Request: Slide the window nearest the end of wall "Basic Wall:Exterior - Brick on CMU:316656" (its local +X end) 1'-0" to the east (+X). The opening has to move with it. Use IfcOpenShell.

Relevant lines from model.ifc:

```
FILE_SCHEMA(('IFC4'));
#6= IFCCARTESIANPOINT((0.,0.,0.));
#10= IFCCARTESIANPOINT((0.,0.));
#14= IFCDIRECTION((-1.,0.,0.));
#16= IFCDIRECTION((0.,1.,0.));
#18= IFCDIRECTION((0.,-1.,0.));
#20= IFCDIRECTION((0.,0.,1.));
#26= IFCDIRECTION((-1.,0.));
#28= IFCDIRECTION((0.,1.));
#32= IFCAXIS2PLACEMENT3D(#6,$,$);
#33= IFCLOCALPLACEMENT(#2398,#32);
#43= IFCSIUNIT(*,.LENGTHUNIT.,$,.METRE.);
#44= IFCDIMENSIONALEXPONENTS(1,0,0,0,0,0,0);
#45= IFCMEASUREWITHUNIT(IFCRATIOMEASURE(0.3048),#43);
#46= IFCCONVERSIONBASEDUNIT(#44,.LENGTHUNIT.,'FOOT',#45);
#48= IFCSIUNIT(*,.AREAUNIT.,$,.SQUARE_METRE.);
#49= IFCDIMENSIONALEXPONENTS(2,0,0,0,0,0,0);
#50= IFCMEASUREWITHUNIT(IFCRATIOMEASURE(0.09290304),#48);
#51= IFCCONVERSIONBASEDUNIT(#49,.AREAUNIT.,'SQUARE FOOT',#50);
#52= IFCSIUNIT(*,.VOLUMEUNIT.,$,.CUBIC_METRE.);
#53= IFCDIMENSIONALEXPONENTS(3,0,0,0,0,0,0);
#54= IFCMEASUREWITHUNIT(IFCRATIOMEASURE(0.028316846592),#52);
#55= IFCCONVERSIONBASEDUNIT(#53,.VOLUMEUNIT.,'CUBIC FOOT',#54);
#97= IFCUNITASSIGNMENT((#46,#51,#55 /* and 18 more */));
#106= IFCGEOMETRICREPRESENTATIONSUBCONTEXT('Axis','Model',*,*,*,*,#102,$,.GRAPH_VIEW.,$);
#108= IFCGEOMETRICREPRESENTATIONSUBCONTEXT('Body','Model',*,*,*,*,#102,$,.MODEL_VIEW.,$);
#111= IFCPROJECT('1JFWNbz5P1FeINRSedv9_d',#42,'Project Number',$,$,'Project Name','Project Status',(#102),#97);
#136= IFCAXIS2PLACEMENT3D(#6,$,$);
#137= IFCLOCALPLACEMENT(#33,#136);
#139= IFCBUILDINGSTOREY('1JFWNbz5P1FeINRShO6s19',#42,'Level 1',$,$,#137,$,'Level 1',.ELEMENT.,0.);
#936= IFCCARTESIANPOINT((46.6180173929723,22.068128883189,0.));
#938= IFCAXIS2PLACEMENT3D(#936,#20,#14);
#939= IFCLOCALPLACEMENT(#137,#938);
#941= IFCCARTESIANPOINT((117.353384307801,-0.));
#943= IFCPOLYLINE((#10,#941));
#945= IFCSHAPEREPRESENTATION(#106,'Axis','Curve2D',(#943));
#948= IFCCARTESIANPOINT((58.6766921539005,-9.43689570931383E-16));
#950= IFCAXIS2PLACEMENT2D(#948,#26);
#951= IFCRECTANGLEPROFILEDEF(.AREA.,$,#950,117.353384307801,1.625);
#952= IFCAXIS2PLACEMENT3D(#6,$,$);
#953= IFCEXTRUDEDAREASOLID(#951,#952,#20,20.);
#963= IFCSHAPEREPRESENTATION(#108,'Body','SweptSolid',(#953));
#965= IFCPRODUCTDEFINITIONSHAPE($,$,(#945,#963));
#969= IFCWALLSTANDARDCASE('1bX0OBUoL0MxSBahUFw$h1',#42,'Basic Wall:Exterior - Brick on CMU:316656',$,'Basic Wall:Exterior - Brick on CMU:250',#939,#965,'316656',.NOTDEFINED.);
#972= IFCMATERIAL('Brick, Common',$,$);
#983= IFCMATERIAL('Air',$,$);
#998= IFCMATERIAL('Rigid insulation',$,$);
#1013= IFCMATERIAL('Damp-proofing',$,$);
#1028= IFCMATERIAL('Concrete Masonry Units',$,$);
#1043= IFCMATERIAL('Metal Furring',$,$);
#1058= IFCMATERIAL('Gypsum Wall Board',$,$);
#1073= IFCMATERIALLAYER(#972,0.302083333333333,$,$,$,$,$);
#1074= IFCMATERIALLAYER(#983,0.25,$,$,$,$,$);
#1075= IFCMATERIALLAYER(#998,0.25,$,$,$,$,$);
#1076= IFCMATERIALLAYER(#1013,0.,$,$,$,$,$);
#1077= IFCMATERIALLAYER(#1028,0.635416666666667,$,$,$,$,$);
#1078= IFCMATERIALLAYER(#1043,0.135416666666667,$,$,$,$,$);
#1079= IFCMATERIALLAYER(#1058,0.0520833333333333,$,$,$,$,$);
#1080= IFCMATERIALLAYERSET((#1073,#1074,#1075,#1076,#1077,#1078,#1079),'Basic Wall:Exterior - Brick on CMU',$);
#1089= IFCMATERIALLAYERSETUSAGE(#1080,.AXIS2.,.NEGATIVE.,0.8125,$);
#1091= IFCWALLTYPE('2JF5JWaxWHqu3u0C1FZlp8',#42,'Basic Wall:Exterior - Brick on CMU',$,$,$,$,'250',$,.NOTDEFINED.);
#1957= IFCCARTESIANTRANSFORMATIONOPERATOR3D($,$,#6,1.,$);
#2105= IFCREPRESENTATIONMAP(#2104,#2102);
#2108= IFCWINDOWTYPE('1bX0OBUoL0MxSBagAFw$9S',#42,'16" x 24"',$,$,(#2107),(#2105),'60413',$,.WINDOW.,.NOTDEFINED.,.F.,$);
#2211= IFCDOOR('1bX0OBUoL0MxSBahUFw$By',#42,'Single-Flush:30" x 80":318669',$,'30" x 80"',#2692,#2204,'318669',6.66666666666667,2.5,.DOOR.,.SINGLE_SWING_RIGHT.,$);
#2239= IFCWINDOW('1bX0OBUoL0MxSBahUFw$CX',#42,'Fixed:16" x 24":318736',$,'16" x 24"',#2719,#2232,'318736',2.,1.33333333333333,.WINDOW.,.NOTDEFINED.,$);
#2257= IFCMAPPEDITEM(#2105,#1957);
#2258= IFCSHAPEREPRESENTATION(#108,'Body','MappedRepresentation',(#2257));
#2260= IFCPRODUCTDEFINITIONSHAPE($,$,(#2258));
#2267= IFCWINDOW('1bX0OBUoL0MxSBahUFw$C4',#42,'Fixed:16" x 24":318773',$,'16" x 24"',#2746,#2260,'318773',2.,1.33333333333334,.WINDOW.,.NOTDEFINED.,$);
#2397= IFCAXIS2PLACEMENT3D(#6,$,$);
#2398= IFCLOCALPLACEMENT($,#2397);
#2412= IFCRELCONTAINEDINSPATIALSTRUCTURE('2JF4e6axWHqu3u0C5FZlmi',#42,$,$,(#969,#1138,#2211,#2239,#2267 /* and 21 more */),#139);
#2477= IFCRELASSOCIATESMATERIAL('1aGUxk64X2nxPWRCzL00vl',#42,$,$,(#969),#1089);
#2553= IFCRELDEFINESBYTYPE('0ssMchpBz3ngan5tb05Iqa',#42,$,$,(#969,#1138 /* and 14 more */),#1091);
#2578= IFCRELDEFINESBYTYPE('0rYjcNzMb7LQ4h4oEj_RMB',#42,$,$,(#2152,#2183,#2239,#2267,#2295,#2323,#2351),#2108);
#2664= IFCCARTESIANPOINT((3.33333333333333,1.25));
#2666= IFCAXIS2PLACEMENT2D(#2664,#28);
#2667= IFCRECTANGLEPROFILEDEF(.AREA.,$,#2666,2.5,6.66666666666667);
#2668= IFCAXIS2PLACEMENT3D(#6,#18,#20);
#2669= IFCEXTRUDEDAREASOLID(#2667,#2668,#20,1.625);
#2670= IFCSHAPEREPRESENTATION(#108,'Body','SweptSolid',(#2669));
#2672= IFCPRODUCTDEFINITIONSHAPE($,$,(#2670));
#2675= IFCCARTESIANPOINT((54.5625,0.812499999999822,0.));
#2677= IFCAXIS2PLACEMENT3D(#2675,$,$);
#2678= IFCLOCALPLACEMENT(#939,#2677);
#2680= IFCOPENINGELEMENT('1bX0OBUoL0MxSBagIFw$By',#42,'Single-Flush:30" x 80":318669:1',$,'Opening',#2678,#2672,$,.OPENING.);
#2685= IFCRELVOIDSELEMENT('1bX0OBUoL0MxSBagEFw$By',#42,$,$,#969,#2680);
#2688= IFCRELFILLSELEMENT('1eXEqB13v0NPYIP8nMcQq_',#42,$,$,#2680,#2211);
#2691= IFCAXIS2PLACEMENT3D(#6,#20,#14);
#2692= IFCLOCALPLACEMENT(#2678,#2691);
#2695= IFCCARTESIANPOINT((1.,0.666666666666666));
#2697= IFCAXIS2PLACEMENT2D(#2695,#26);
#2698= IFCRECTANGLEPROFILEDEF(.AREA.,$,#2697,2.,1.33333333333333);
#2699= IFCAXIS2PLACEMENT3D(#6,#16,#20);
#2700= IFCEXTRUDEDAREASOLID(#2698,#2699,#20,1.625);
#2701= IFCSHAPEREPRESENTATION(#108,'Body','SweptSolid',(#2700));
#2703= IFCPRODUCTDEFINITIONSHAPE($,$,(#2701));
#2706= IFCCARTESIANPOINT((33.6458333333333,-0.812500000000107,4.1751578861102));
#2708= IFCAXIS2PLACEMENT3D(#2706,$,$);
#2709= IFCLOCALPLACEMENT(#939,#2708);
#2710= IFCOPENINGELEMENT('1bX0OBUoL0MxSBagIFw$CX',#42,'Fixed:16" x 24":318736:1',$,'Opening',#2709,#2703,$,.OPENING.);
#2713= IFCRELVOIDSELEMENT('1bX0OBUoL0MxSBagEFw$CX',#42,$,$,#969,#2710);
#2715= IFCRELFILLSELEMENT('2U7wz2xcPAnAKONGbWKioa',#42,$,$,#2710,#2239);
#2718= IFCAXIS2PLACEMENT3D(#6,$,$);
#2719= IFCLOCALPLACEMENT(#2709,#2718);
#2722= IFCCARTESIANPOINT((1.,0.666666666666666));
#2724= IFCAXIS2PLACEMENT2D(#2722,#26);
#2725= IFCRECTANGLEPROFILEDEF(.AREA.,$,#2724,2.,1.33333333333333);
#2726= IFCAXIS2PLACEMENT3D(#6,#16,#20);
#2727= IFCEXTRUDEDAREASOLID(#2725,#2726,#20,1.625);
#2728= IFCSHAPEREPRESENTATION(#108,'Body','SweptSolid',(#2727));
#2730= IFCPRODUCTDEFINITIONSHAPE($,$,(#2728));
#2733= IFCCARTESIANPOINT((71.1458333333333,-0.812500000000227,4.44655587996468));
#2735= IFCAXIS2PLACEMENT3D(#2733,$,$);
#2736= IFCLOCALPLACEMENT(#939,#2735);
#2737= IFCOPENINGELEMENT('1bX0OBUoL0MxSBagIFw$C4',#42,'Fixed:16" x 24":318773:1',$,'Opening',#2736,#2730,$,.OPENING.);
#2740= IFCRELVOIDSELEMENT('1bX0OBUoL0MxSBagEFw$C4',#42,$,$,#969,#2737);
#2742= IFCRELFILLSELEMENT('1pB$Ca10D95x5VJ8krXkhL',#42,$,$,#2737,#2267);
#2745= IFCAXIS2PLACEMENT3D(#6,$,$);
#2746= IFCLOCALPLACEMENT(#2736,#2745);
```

```python
import ifcopenshell
import ifcopenshell.api.geometry
import ifcopenshell.util.placement
import ifcopenshell.util.unit

model = ifcopenshell.open("model.ifc")
unit_scale = ifcopenshell.util.unit.calculate_unit_scale(model)

window = model.by_guid("1bX0OBUoL0MxSBahUFw$C4")
opening = window.FillsVoids[0].RelatingOpeningElement
wall = opening.VoidsElements[0].RelatingBuildingElement

wall_matrix = ifcopenshell.util.placement.get_local_placement(wall.ObjectPlacement)
shift = wall_matrix[:3, 0] * -12 * 0.0254 / unit_scale
before = ifcopenshell.util.placement.get_local_placement(window.ObjectPlacement)[:3, 3].copy()

# The window is placed relative to its opening, so it follows when the opening moves.
matrix = ifcopenshell.util.placement.get_local_placement(opening.ObjectPlacement)
matrix[:3, 3] += shift
ifcopenshell.api.geometry.edit_object_placement(
    model, product=opening, matrix=matrix, is_si=False, should_transform_children=True
)

after = ifcopenshell.util.placement.get_local_placement(window.ObjectPlacement)[:3, 3]
print("window moved by", (after - before).round(3) + 0.0)

model.write("model_v2.ifc")
```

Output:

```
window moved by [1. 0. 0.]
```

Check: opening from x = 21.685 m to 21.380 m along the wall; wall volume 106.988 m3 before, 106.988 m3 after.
